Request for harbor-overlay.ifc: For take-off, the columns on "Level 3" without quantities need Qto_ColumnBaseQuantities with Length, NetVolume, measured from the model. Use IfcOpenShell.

First a look at what the model holds.

```python
import ifcopenshell
import ifcopenshell.util.element
import ifcopenshell.util.unit

model = ifcopenshell.open("harbor-overlay.ifc")
print(model.schema)
for unit_type in ("LENGTHUNIT", "AREAUNIT", "VOLUMEUNIT"):
    print(unit_type, ifcopenshell.util.unit.calculate_unit_scale(model, unit_type))
storey = next(s for s in model.by_type("IfcBuildingStorey") if s.Name == "Level 3")
columns = [e for e in ifcopenshell.util.element.get_decomposition(storey) if e.is_a("IfcColumn")]
for e in sorted(columns, key=lambda e: e.id()):
    print(e.id(), e.is_a(), e.Name, list(ifcopenshell.util.element.get_psets(e, qtos_only=True)), sep=" | ")
```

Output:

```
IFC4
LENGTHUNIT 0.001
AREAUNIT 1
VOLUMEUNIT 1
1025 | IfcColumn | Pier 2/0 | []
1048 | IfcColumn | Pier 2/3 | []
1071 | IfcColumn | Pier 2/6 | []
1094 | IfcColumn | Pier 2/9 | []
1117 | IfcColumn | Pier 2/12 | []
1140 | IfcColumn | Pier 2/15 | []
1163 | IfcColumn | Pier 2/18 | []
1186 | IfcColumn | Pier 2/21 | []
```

```python
import ifcopenshell
import ifcopenshell.api.pset
import ifcopenshell.geom
import ifcopenshell.util.element
import ifcopenshell.util.shape
import ifcopenshell.util.unit

model = ifcopenshell.open("harbor-overlay.ifc")
unit_scale = ifcopenshell.util.unit.calculate_unit_scale(model)
volume_scale = ifcopenshell.util.unit.calculate_unit_scale(model, "VOLUMEUNIT")
settings = ifcopenshell.geom.settings()

storey = next(s for s in model.by_type("IfcBuildingStorey") if s.Name == "Level 3")
columns = [e for e in ifcopenshell.util.element.get_decomposition(storey) if e.is_a("IfcColumn")]

for e in sorted(columns, key=lambda e: e.id()):
    if ifcopenshell.util.element.get_psets(e, qtos_only=True, should_inherit=False):
        continue
    # Geometry comes back in metres, in the element's own axes.
    shape = ifcopenshell.geom.create_shape(settings, e)
    values = {
        "Length": ifcopenshell.util.shape.get_z(shape.geometry) / unit_scale,
        "NetVolume": ifcopenshell.util.shape.get_volume(shape.geometry) / volume_scale,
    }
    qto = ifcopenshell.api.pset.add_qto(model, product=e, name="Qto_ColumnBaseQuantities")
    ifcopenshell.api.pset.edit_qto(model, qto=qto, properties=values)
    print(e.id(), {k: round(v, 3) for k, v in values.items()})

model.write("harbor-overlay_v2.ifc")
```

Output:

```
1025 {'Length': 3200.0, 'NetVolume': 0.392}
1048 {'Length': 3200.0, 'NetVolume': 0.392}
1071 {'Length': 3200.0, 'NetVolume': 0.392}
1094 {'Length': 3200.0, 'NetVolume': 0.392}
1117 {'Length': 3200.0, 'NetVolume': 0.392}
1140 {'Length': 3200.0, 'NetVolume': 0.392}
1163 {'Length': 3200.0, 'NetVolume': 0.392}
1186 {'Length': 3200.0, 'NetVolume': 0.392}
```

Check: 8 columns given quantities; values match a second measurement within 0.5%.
